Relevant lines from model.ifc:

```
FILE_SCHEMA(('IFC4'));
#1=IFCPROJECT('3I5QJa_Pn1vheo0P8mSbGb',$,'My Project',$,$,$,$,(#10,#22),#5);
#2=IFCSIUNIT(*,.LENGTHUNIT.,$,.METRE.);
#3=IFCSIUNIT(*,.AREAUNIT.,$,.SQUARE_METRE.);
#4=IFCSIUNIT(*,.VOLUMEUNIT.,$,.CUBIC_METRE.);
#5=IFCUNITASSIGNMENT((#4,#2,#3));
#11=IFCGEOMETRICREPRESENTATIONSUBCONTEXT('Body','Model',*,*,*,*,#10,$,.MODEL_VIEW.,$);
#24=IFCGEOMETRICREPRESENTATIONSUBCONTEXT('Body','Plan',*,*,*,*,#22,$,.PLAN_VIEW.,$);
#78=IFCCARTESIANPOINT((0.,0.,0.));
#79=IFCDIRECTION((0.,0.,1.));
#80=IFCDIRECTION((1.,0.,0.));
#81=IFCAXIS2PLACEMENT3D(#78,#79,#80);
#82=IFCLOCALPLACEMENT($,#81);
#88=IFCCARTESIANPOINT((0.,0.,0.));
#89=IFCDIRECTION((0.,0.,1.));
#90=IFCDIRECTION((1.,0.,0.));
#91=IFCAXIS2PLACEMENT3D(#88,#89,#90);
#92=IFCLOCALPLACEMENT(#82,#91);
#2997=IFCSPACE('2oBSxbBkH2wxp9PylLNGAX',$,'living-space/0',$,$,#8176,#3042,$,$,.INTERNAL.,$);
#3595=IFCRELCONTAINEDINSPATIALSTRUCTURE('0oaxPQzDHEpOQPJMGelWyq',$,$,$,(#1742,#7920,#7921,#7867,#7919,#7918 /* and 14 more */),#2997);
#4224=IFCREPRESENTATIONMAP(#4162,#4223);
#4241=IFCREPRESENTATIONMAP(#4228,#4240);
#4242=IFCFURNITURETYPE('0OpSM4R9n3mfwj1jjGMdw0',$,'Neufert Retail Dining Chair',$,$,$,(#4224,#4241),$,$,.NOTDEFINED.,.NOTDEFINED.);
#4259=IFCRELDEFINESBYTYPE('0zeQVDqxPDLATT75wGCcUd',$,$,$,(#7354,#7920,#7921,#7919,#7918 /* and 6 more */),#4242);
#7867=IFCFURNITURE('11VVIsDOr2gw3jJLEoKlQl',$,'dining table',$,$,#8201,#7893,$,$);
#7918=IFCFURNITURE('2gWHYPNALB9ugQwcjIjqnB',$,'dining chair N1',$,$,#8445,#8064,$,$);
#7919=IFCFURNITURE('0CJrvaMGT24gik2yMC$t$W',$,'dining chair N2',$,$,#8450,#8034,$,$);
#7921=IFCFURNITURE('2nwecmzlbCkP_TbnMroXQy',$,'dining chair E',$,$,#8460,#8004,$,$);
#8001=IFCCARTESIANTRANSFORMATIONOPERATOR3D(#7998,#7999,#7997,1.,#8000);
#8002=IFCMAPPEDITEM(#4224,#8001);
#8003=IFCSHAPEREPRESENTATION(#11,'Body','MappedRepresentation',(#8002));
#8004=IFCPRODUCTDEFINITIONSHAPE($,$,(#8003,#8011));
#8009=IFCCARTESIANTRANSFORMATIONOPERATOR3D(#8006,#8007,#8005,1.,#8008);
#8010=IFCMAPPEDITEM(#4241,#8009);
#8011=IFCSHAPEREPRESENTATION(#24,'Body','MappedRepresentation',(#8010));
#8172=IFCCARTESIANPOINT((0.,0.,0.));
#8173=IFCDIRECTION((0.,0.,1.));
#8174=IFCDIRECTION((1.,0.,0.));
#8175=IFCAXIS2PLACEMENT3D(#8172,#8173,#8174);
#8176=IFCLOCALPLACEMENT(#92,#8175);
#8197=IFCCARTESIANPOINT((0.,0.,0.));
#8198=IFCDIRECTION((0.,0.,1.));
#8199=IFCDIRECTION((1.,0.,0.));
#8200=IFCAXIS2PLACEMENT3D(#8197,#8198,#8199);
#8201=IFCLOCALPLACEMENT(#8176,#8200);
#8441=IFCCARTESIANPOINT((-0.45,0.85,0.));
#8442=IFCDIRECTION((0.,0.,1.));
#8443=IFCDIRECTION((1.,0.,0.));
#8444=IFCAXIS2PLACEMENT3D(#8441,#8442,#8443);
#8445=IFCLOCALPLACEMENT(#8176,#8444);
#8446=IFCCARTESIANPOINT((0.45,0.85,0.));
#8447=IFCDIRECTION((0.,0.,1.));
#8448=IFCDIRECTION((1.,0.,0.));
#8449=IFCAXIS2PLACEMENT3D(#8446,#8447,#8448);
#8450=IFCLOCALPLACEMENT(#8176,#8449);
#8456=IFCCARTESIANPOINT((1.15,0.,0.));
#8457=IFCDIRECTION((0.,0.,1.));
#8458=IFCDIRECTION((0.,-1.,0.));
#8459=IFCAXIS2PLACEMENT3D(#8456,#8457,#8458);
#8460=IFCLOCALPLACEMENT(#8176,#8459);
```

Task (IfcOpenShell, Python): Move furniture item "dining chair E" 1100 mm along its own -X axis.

```python
import ifcopenshell
import ifcopenshell.api.geometry
import ifcopenshell.util.placement

model = ifcopenshell.open("model.ifc")

item = model.by_guid("2nwecmzlbCkP_TbnMroXQy")
matrix = ifcopenshell.util.placement.get_local_placement(item.ObjectPlacement)
matrix[:3, 3] -= matrix[:3, 0] * 1.1
ifcopenshell.api.geometry.edit_object_placement(model, product=item, matrix=matrix, is_si=False)

print(ifcopenshell.util.placement.get_local_placement(item.ObjectPlacement).round(3) + 0.0)

model.write("model_edited.ifc")
```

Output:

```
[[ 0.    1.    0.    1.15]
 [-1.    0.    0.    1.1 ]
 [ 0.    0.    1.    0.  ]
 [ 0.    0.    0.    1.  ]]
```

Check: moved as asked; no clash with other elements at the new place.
